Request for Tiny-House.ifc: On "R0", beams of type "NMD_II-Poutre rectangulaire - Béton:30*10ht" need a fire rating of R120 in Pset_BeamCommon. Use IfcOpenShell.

First a look at what the model holds.

```python
import ifcopenshell
import ifcopenshell.util.element

model = ifcopenshell.open("Tiny-House.ifc")
print(model.schema)
storey = next(s for s in model.by_type("IfcBuildingStorey") if s.Name == "R0")
beams = [e for e in ifcopenshell.util.element.get_decomposition(storey) if e.is_a("IfcBeam")]
seen = {}
for e in beams:
    element_type = ifcopenshell.util.element.get_type(e)
    key = (element_type.Name if element_type != e and element_type else None, ifcopenshell.util.element.get_pset(e, "Pset_BeamCommon", "FireRating"))
    seen[key] = seen.get(key, 0) + 1
for (name, value), count in sorted(seen.items(), key=str):
    print(count, "x", name, "|", value)
```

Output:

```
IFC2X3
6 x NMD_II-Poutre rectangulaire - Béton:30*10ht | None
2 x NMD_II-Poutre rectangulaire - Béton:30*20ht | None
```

```python
import ifcopenshell
import ifcopenshell.api.pset
import ifcopenshell.util.element

model = ifcopenshell.open("Tiny-House.ifc")

storey = next(s for s in model.by_type("IfcBuildingStorey") if s.Name == "R0")
beams = [e for e in ifcopenshell.util.element.get_decomposition(storey) if e.is_a("IfcBeam")]

count = 0
for e in beams:
    element_type = ifcopenshell.util.element.get_type(e)
    if element_type in (None, e) or element_type.Name != "NMD_II-Poutre rectangulaire - Béton:30*10ht":
        continue
    # add_pset returns the element's existing set when there is one.
    pset = ifcopenshell.api.pset.add_pset(model, product=e, name="Pset_BeamCommon")
    ifcopenshell.api.pset.edit_pset(model, pset=pset, properties={"FireRating": "R120"})
    count += 1

print(count, "beams updated")

model.write("Tiny-House_v2.ifc")
```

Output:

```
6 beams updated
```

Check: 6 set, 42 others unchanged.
